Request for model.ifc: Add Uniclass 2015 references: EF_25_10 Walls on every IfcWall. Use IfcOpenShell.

First a look at what the model holds.

```python
import ifcopenshell

model = ifcopenshell.open("model.ifc")
print(model.schema)
print("classifications:", [c.Name for c in model.by_type("IfcClassification")])
for ifc_class in ("IfcDoor", "IfcRoof", "IfcStair", "IfcWall", "IfcWindow"):
    print(ifc_class, len(model.by_type(ifc_class)))
```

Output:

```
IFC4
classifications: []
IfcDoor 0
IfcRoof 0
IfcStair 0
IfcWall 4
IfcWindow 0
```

```python
import ifcopenshell
import ifcopenshell.api.classification

model = ifcopenshell.open("model.ifc")

system = ifcopenshell.api.classification.add_classification(model, classification="Uniclass 2015")

codes = {
    "IfcWall": ("EF_25_10", "Walls"),
}
for ifc_class, (code, name) in codes.items():
    products = model.by_type(ifc_class)
    ifcopenshell.api.classification.add_reference(
        model, products=products, classification=system, identification=code, name=name
    )
    print(code, len(products))

model.write("model_updated.ifc")
```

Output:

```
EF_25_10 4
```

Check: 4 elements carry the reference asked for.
